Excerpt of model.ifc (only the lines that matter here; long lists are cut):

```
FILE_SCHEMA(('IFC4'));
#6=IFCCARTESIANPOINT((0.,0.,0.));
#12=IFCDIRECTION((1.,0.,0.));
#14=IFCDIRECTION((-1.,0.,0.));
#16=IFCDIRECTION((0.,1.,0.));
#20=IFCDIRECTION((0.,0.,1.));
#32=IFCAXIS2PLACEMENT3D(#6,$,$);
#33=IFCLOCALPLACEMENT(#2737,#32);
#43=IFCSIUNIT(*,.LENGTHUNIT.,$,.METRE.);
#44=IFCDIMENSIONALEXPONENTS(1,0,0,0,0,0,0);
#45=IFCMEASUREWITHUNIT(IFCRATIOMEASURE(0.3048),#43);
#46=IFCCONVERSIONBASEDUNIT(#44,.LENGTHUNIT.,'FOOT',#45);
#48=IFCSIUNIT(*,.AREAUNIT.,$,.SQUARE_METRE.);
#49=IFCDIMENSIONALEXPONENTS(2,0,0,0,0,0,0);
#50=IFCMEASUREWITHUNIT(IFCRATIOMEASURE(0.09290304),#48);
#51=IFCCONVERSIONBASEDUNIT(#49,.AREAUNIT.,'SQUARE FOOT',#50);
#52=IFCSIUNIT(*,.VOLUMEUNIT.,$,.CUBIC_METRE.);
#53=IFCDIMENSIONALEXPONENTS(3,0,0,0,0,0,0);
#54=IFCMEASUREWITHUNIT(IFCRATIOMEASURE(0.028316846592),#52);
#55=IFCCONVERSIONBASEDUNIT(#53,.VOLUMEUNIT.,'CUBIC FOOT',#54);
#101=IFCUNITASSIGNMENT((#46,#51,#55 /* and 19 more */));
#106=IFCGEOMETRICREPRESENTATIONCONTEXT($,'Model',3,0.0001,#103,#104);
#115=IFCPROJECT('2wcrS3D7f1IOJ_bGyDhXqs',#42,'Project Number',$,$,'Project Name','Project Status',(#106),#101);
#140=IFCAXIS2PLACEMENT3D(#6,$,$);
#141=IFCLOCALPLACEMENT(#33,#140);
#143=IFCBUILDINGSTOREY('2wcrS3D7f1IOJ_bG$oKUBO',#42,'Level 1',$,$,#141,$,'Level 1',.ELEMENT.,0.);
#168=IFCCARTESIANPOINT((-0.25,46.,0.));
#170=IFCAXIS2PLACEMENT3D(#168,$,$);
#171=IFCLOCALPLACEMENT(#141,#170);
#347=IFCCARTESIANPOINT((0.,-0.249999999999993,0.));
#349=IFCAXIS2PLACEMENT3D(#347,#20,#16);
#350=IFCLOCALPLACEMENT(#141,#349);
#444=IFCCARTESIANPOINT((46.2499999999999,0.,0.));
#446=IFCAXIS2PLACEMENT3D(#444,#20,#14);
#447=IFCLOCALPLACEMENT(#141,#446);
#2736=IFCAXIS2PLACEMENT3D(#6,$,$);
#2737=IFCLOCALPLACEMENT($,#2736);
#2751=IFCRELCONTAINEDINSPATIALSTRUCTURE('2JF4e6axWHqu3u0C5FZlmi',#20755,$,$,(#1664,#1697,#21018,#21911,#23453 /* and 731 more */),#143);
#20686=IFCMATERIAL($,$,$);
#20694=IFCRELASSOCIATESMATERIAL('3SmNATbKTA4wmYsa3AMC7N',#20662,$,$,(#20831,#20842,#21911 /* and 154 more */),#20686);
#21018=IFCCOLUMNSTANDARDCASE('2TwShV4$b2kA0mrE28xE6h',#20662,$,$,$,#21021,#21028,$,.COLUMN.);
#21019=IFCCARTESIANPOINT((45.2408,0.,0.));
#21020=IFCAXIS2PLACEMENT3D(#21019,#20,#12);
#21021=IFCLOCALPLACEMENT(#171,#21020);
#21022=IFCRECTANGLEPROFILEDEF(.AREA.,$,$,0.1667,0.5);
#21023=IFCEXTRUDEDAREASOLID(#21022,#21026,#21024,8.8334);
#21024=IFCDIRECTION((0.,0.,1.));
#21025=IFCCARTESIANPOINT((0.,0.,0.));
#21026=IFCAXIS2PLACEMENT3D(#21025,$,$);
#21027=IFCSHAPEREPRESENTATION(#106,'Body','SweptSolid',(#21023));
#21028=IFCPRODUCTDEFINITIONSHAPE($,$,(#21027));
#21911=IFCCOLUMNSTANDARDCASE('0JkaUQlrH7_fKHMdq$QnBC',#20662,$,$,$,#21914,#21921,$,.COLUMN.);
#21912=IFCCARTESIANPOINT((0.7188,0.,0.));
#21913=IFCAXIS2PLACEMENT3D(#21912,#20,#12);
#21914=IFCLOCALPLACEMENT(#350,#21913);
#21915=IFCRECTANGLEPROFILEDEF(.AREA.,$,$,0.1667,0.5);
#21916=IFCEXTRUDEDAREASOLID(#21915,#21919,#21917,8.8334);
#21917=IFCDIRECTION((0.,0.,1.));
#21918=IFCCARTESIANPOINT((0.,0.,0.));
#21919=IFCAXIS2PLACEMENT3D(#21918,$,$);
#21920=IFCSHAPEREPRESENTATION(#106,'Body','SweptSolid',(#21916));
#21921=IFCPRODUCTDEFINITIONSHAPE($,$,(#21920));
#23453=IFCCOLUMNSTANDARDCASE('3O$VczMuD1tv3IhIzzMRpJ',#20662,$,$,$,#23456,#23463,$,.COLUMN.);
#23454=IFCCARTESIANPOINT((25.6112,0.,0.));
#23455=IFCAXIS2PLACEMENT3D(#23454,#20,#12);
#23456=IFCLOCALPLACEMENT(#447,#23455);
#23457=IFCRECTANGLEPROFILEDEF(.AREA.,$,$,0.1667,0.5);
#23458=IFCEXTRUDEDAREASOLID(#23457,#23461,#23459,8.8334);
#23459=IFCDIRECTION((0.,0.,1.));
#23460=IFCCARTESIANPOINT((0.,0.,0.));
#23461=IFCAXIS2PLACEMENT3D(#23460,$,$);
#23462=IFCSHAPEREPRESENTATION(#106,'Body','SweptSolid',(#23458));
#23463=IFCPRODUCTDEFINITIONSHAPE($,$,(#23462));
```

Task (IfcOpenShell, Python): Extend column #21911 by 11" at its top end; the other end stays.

```python
import ifcopenshell
import ifcopenshell.util.unit

model = ifcopenshell.open("model.ifc")
unit_scale = ifcopenshell.util.unit.calculate_unit_scale(model)

member = model.by_guid("0JkaUQlrH7_fKHMdq$QnBC")
change = 11 * 0.0254 / unit_scale

# The extrusion runs towards the end named, so only its depth changes.
body = next(r for r in member.Representation.Representations if r.RepresentationIdentifier == "Body")
solid = body.Items[0]
old_length = solid.Depth
solid.Depth += change

print(f"length {old_length:g} -> {solid.Depth:g}")

model.write("model_updated.ifc")
```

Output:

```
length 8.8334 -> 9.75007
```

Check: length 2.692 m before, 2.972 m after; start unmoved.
